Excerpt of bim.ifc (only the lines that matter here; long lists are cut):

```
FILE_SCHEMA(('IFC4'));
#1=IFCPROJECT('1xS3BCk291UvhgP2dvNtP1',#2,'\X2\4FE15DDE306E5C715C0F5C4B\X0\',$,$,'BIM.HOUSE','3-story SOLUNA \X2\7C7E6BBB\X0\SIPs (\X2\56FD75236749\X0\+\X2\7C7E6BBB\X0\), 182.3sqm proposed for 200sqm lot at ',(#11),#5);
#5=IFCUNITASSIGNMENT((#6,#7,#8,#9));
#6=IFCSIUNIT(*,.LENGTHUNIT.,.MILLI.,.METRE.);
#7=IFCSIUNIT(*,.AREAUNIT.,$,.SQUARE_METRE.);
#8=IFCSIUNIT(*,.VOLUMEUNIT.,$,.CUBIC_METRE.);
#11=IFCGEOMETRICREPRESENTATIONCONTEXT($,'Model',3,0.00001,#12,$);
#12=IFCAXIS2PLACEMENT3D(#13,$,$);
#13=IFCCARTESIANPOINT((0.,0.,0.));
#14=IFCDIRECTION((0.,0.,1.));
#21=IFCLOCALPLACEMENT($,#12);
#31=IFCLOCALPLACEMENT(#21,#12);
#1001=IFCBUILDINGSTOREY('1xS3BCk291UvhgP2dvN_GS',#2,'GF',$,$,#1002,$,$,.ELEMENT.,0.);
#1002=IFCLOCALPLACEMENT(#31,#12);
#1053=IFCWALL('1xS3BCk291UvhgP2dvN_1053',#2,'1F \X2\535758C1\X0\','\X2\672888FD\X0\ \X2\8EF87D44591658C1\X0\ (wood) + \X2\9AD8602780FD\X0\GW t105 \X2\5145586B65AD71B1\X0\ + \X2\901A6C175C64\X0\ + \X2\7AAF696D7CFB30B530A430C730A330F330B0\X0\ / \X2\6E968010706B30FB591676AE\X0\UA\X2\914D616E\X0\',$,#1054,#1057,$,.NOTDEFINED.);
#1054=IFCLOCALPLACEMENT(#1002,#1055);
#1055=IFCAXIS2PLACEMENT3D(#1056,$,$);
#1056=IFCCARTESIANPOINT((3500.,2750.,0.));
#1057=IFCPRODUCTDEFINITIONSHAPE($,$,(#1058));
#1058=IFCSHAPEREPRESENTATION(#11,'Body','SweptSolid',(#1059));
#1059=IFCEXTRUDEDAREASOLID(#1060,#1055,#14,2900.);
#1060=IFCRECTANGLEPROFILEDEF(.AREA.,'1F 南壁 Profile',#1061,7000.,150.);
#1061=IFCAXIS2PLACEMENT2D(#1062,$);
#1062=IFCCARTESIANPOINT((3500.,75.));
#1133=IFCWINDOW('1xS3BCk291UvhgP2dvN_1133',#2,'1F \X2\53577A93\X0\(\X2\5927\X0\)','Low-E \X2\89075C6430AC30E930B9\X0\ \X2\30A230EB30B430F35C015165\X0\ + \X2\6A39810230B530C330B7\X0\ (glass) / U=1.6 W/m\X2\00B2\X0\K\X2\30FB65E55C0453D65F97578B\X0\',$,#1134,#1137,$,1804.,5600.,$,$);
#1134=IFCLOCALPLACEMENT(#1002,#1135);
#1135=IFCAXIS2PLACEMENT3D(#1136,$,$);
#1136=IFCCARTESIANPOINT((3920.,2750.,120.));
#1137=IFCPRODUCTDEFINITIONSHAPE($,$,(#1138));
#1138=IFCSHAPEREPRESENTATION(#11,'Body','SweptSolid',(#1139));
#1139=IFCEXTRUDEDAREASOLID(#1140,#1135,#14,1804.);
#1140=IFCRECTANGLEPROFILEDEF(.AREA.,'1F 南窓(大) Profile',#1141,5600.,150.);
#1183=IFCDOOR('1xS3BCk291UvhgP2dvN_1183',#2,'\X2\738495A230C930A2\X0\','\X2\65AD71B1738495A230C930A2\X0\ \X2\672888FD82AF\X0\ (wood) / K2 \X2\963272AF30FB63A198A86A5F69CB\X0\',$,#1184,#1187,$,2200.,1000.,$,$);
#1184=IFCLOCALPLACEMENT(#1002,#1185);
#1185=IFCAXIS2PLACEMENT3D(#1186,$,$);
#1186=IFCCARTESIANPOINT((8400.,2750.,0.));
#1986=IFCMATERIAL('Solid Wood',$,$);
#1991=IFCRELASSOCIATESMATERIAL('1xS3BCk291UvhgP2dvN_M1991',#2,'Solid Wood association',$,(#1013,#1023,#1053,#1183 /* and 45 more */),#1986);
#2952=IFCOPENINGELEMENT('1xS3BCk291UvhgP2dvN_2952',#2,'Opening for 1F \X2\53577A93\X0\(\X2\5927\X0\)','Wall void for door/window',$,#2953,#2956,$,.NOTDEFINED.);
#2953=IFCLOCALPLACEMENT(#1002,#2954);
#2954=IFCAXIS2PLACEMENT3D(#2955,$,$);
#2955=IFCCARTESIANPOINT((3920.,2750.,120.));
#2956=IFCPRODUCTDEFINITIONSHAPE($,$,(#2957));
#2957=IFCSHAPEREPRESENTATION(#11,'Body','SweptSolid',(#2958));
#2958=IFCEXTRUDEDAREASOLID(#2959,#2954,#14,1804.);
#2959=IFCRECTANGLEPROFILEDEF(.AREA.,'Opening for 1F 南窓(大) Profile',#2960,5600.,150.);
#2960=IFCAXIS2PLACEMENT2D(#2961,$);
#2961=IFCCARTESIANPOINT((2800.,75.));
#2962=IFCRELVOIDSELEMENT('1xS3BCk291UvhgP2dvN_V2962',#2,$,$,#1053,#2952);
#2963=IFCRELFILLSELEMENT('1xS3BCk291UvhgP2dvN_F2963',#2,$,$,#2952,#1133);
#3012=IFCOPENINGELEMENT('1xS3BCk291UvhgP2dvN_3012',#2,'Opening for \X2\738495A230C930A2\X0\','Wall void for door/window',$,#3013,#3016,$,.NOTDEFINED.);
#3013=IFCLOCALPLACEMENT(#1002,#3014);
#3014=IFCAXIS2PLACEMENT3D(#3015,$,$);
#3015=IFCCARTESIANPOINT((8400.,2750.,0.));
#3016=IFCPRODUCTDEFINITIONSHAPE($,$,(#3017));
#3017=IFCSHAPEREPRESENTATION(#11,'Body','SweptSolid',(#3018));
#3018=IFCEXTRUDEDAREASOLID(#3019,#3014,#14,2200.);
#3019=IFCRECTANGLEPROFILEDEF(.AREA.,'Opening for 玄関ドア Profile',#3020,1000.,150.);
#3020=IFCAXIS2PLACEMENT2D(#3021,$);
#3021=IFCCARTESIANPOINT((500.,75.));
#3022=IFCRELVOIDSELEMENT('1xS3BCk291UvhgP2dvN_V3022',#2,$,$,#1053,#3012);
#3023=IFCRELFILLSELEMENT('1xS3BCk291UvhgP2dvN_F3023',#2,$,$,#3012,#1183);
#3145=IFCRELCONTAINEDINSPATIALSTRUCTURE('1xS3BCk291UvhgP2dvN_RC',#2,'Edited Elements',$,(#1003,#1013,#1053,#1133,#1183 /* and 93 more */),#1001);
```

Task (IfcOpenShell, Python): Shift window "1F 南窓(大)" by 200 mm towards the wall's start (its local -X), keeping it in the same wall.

```python
import ifcopenshell
import ifcopenshell.api.geometry
import ifcopenshell.util.placement

model = ifcopenshell.open("bim.ifc")

window = model.by_guid("1xS3BCk291UvhgP2dvN_1133")
opening = window.FillsVoids[0].RelatingOpeningElement
wall = opening.VoidsElements[0].RelatingBuildingElement

wall_matrix = ifcopenshell.util.placement.get_local_placement(wall.ObjectPlacement)
shift = wall_matrix[:3, 0] * -200.0
before = ifcopenshell.util.placement.get_local_placement(window.ObjectPlacement)[:3, 3].copy()

# The window is not placed relative to its opening, so move both.
for product in (opening, window):
    matrix = ifcopenshell.util.placement.get_local_placement(product.ObjectPlacement)
    matrix[:3, 3] += shift
    ifcopenshell.api.geometry.edit_object_placement(model, product=product, matrix=matrix, is_si=False)

after = ifcopenshell.util.placement.get_local_placement(window.ObjectPlacement)[:3, 3]
print("window moved by", (after - before).round(3) + 0.0)

model.write("bim_rev.ifc")
```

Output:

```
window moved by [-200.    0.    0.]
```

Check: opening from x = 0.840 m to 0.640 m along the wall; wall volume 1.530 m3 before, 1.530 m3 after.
